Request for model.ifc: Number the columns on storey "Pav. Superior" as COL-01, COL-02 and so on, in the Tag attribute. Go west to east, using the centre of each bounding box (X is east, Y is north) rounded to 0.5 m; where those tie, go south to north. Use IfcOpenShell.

First a look at what the model holds.

```python
import ifcopenshell
import ifcopenshell.util.element
import ifcopenshell.util.placement

model = ifcopenshell.open("model.ifc")
print(model.schema)
storey = next(s for s in model.by_type("IfcBuildingStorey") if s.Name == "Pav. Superior")
columns = [e for e in ifcopenshell.util.element.get_decomposition(storey) if e.is_a("IfcColumn")]
for e in sorted(columns, key=lambda e: e.id()):
    origin = ifcopenshell.util.placement.get_local_placement(e.ObjectPlacement)[:3, 3]
    print(e.id(), e.Tag, e.Name, origin.round(2) + 0.0, sep=" | ")
```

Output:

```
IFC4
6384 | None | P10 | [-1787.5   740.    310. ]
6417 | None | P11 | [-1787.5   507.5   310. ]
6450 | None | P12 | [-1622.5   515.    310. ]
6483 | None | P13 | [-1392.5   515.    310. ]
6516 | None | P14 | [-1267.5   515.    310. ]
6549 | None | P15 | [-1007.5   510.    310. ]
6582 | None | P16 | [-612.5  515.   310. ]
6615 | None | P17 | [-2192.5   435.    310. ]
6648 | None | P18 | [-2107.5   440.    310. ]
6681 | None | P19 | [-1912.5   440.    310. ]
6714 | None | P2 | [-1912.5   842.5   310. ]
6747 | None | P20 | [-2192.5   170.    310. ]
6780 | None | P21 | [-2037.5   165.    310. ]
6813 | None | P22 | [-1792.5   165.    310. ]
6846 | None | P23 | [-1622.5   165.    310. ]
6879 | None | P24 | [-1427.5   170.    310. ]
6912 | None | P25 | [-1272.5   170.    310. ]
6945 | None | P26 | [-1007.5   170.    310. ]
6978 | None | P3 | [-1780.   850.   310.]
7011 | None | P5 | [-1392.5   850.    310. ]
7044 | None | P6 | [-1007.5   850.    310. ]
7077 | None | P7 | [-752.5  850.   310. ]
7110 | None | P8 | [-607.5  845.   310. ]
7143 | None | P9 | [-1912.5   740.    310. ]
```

```python
import ifcopenshell
import ifcopenshell.geom
import ifcopenshell.util.element
import ifcopenshell.util.shape

model = ifcopenshell.open("model.ifc")
settings = ifcopenshell.geom.settings()
settings.set("use-world-coords", True)


def centre(element):
    shape = ifcopenshell.geom.create_shape(settings, element)
    return ifcopenshell.util.shape.get_bbox_centroid(shape.geometry)


storey = next(s for s in model.by_type("IfcBuildingStorey") if s.Name == "Pav. Superior")
columns = [e for e in ifcopenshell.util.element.get_decomposition(storey) if e.is_a("IfcColumn")]

# Insertion points can sit at a corner or the storey origin, so sort by the geometry (in metres).
centres = {e: centre(e) for e in columns}
columns.sort(key=lambda e: (round(centres[e][0] / 0.5), centres[e][1]))

for i, e in enumerate(columns, start=1):
    number = f"COL-{i:02d}"
    e.Tag = number
    print(e.id(), number)

model.write("model_updated.ifc")
```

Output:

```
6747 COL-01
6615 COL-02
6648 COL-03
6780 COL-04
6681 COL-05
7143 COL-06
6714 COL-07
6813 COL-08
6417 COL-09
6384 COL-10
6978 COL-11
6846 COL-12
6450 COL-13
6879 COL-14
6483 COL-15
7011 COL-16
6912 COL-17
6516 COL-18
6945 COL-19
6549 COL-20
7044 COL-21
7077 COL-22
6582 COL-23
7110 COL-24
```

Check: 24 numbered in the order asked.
